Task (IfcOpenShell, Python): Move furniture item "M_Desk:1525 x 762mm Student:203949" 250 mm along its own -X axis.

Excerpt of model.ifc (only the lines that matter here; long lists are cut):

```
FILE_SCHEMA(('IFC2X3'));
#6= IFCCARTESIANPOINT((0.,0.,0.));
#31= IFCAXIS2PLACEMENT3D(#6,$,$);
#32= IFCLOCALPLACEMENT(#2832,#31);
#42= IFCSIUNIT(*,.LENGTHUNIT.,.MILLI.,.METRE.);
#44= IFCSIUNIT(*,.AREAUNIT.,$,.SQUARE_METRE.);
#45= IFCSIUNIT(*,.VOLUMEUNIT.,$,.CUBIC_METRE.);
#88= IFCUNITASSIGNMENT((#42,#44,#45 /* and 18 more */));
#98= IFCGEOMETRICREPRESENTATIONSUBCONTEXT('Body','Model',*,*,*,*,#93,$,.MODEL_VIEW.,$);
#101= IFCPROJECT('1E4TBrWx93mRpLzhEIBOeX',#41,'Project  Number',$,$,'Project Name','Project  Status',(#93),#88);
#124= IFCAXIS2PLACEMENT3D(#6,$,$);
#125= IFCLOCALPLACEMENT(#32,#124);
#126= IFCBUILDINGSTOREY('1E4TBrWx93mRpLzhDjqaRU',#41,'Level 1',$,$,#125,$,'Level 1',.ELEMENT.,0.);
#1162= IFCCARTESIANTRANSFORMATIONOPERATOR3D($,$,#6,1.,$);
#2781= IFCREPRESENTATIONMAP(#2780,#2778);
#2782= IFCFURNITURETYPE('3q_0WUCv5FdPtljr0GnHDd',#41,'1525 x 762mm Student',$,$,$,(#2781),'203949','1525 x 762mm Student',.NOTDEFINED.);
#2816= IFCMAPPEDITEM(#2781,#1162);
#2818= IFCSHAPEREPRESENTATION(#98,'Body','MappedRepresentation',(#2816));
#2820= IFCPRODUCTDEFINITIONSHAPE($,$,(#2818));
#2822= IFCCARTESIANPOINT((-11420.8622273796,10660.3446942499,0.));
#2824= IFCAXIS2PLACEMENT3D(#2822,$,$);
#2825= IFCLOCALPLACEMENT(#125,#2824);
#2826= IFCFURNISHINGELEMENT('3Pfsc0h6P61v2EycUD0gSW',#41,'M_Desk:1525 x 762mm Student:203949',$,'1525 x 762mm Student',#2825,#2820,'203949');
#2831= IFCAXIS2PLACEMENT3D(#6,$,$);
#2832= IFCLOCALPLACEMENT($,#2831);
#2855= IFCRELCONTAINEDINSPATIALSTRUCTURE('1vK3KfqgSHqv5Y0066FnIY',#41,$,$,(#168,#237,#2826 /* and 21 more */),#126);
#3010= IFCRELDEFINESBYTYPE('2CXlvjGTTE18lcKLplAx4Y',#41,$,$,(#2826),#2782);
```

```python
import ifcopenshell
import ifcopenshell.api.geometry
import ifcopenshell.util.placement

model = ifcopenshell.open("model.ifc")

item = model.by_guid("3Pfsc0h6P61v2EycUD0gSW")
matrix = ifcopenshell.util.placement.get_local_placement(item.ObjectPlacement)
matrix[:3, 3] -= matrix[:3, 0] * 250.0
ifcopenshell.api.geometry.edit_object_placement(model, product=item, matrix=matrix, is_si=False)

print(ifcopenshell.util.placement.get_local_placement(item.ObjectPlacement).round(3) + 0.0)

model.write("model_edited.ifc")
```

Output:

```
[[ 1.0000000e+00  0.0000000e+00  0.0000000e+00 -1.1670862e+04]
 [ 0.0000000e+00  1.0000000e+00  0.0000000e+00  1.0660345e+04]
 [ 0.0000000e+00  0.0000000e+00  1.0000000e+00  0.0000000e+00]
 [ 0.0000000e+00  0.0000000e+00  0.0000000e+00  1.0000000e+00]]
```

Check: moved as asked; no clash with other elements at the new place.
